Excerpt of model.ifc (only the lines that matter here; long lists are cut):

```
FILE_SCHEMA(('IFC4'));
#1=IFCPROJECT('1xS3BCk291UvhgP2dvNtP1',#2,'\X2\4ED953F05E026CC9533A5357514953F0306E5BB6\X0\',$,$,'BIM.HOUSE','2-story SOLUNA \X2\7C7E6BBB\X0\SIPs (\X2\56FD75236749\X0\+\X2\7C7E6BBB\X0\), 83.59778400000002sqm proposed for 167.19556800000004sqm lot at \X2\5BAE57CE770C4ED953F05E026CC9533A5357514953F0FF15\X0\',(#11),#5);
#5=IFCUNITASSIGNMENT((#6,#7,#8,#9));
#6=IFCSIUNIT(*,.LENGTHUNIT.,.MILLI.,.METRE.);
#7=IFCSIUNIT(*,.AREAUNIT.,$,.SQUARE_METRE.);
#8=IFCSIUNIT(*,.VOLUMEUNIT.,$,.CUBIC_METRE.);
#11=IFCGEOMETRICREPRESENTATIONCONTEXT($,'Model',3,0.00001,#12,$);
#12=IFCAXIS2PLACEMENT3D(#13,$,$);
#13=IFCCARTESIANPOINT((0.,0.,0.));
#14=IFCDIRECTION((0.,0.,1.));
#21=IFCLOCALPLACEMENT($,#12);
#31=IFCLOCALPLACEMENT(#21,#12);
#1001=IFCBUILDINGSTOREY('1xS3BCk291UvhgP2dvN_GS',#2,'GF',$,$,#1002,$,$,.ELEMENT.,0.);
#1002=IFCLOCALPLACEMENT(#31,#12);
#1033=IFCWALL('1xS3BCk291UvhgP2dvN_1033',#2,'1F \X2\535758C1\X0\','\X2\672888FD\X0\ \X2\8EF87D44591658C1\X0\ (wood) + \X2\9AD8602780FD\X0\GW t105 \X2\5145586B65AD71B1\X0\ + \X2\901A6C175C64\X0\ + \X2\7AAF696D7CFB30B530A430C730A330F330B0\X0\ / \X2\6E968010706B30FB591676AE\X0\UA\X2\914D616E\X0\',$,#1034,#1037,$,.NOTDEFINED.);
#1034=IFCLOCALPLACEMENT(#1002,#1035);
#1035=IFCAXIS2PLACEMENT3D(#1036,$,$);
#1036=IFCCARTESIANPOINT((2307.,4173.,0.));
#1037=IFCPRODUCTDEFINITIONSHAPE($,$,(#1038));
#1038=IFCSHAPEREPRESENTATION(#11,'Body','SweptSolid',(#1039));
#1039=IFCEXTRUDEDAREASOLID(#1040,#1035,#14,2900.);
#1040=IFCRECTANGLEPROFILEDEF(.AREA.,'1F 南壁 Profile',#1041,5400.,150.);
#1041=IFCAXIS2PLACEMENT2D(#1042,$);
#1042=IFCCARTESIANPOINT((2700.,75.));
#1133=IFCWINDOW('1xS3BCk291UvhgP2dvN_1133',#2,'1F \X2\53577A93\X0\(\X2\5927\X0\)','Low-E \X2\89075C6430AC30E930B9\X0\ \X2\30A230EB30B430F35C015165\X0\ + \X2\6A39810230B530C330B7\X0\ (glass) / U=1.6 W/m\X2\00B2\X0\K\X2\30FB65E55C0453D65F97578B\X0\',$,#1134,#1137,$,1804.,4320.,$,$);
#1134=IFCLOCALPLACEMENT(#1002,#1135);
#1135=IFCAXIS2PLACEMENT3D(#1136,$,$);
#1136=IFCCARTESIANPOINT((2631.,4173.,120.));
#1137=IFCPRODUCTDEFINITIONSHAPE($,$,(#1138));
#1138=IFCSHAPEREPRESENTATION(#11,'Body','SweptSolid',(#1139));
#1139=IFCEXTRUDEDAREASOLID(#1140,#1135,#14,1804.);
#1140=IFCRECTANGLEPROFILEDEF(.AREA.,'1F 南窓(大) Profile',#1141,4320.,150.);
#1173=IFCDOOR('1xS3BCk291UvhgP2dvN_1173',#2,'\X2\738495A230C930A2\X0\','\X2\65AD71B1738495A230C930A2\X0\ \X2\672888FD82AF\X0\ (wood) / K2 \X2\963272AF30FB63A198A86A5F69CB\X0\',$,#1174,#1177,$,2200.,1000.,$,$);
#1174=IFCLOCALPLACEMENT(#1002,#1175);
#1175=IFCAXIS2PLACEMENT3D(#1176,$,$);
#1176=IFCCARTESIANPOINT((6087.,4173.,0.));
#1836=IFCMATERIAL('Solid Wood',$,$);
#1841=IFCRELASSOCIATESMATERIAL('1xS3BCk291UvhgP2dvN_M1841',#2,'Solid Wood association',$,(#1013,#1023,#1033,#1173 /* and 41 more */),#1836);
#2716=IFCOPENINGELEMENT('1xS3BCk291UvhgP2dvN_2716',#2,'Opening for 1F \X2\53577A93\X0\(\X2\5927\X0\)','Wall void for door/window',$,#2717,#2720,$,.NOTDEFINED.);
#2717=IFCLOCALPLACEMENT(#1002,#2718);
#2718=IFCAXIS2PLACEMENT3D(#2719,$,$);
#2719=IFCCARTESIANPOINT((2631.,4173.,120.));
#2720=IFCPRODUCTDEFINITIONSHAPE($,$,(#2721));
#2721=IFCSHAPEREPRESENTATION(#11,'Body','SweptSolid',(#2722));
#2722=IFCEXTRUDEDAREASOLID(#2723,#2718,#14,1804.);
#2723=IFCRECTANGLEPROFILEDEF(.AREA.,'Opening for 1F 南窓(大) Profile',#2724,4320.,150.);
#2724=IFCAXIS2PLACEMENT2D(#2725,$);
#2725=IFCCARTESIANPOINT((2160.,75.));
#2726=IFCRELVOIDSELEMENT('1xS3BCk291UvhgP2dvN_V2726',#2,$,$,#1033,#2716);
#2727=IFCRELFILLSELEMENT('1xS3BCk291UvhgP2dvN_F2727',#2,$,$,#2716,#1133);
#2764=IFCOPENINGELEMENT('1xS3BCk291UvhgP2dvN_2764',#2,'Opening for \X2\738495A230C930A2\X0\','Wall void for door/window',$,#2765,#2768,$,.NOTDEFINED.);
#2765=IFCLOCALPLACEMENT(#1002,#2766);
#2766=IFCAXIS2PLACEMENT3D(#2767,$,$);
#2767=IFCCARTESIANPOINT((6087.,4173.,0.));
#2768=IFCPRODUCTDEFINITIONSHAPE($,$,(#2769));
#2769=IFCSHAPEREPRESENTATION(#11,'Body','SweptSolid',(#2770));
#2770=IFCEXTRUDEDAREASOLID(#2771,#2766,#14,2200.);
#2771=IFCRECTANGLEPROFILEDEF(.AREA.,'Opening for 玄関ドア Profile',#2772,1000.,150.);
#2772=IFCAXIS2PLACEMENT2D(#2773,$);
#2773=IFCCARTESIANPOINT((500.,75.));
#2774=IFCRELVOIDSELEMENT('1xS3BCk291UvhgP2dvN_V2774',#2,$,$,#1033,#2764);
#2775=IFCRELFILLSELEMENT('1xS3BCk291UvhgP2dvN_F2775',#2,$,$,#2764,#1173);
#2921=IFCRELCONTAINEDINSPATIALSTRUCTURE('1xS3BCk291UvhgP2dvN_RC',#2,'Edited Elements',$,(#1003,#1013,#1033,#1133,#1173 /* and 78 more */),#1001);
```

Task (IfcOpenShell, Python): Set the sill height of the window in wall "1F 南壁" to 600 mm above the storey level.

```python
import numpy as np
import ifcopenshell
import ifcopenshell.api.geometry
import ifcopenshell.geom
import ifcopenshell.util.element
import ifcopenshell.util.placement
import ifcopenshell.util.shape
import ifcopenshell.util.unit

model = ifcopenshell.open("model.ifc")
unit_scale = ifcopenshell.util.unit.calculate_unit_scale(model)

window = model.by_guid("1xS3BCk291UvhgP2dvN_1133")
opening = window.FillsVoids[0].RelatingOpeningElement
storey = ifcopenshell.util.element.get_container(window, ifc_class="IfcBuildingStorey")
level = ifcopenshell.util.placement.get_local_placement(storey.ObjectPlacement)[2, 3]

# The opening's origin need not be at the sill, so measure its lowest point.
shape = ifcopenshell.geom.create_shape(ifcopenshell.geom.settings(), opening)
bottom = ifcopenshell.util.shape.get_shape_bottom_elevation(shape, shape.geometry) / unit_scale
dz = level + 0.6 / unit_scale - bottom

shift = np.array([0.0, 0.0, dz])
# The window is not placed relative to its opening, so move both.
for product in (opening, window):
    matrix = ifcopenshell.util.placement.get_local_placement(product.ObjectPlacement)
    matrix[:3, 3] += shift
    ifcopenshell.api.geometry.edit_object_placement(model, product=product, matrix=matrix, is_si=False)

print(f"moved by {dz * unit_scale:+.3f} m")

model.write("model_updated.ifc")
```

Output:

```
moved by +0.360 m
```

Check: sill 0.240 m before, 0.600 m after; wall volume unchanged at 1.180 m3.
